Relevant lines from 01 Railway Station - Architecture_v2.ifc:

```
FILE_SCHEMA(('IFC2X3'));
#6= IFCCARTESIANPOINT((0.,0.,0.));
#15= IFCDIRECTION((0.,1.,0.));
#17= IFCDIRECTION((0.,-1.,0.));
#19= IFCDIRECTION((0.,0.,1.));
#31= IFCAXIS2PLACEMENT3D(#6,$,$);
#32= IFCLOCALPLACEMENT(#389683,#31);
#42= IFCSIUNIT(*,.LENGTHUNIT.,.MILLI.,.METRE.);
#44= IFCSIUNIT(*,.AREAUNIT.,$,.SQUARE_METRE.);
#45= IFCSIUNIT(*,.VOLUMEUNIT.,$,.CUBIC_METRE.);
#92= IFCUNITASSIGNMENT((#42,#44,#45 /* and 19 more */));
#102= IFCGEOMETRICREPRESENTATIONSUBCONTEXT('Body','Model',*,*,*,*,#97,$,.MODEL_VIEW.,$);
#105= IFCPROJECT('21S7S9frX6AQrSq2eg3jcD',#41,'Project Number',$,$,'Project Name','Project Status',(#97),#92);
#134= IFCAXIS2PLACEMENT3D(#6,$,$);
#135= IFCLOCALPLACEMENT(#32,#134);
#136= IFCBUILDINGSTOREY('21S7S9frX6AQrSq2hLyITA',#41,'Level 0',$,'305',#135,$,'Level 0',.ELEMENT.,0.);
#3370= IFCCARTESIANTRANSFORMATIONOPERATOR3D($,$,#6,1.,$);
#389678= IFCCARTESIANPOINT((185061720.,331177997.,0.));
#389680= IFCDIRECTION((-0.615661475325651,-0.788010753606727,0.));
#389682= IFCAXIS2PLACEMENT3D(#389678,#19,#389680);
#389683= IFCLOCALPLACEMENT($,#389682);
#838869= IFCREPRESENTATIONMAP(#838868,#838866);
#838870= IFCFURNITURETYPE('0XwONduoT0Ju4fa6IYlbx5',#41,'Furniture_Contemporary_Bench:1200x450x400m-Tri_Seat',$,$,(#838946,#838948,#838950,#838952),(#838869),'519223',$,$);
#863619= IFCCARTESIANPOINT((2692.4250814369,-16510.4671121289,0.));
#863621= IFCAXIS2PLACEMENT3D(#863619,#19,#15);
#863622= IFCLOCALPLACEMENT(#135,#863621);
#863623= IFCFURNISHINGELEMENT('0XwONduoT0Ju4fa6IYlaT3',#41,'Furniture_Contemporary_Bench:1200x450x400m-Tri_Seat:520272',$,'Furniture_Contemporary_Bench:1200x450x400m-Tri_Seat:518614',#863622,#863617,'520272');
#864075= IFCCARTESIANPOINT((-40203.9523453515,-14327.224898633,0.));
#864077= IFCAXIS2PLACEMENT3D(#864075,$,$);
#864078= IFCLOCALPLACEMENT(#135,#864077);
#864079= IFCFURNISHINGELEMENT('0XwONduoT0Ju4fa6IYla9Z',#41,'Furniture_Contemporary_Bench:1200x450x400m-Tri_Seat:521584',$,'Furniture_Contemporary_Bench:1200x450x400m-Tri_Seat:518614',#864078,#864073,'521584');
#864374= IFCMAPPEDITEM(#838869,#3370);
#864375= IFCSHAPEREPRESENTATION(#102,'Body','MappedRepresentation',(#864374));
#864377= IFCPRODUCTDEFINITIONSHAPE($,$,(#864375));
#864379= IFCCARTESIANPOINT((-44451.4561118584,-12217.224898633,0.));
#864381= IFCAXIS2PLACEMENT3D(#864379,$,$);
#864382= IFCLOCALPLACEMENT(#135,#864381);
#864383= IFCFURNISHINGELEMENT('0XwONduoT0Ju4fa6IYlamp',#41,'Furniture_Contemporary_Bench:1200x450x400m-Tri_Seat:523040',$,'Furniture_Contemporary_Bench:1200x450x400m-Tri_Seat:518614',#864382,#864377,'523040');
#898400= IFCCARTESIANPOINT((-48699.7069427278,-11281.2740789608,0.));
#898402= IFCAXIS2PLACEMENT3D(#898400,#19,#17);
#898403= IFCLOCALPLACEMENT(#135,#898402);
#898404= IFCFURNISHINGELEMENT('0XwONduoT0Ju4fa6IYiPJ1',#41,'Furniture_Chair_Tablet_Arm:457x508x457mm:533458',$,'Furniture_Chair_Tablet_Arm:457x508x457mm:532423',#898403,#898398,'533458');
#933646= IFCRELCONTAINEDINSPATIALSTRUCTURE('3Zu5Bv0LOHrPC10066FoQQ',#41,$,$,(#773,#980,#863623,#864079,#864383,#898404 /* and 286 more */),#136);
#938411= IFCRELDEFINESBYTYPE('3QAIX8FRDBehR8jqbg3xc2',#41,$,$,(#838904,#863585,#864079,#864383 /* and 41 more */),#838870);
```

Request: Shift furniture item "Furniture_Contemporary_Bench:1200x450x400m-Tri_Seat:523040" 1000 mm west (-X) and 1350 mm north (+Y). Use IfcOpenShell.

```python
import ifcopenshell
import ifcopenshell.api.geometry
import ifcopenshell.util.placement

model = ifcopenshell.open("01 Railway Station - Architecture_v2.ifc")

item = model.by_id(864383)
matrix = ifcopenshell.util.placement.get_local_placement(item.ObjectPlacement)
matrix[0, 3] -= 1000.0
matrix[1, 3] += 1350.0
ifcopenshell.api.geometry.edit_object_placement(model, product=item, matrix=matrix, is_si=False)

print(ifcopenshell.util.placement.get_local_placement(item.ObjectPlacement).round(3) + 0.0)

model.write("01 Railway Station - Architecture_v2_rev.ifc")
```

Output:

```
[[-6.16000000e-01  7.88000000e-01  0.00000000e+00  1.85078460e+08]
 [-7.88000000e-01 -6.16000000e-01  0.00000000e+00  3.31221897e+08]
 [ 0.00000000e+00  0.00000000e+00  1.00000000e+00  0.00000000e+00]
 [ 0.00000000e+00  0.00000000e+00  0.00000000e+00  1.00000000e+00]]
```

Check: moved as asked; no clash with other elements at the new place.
